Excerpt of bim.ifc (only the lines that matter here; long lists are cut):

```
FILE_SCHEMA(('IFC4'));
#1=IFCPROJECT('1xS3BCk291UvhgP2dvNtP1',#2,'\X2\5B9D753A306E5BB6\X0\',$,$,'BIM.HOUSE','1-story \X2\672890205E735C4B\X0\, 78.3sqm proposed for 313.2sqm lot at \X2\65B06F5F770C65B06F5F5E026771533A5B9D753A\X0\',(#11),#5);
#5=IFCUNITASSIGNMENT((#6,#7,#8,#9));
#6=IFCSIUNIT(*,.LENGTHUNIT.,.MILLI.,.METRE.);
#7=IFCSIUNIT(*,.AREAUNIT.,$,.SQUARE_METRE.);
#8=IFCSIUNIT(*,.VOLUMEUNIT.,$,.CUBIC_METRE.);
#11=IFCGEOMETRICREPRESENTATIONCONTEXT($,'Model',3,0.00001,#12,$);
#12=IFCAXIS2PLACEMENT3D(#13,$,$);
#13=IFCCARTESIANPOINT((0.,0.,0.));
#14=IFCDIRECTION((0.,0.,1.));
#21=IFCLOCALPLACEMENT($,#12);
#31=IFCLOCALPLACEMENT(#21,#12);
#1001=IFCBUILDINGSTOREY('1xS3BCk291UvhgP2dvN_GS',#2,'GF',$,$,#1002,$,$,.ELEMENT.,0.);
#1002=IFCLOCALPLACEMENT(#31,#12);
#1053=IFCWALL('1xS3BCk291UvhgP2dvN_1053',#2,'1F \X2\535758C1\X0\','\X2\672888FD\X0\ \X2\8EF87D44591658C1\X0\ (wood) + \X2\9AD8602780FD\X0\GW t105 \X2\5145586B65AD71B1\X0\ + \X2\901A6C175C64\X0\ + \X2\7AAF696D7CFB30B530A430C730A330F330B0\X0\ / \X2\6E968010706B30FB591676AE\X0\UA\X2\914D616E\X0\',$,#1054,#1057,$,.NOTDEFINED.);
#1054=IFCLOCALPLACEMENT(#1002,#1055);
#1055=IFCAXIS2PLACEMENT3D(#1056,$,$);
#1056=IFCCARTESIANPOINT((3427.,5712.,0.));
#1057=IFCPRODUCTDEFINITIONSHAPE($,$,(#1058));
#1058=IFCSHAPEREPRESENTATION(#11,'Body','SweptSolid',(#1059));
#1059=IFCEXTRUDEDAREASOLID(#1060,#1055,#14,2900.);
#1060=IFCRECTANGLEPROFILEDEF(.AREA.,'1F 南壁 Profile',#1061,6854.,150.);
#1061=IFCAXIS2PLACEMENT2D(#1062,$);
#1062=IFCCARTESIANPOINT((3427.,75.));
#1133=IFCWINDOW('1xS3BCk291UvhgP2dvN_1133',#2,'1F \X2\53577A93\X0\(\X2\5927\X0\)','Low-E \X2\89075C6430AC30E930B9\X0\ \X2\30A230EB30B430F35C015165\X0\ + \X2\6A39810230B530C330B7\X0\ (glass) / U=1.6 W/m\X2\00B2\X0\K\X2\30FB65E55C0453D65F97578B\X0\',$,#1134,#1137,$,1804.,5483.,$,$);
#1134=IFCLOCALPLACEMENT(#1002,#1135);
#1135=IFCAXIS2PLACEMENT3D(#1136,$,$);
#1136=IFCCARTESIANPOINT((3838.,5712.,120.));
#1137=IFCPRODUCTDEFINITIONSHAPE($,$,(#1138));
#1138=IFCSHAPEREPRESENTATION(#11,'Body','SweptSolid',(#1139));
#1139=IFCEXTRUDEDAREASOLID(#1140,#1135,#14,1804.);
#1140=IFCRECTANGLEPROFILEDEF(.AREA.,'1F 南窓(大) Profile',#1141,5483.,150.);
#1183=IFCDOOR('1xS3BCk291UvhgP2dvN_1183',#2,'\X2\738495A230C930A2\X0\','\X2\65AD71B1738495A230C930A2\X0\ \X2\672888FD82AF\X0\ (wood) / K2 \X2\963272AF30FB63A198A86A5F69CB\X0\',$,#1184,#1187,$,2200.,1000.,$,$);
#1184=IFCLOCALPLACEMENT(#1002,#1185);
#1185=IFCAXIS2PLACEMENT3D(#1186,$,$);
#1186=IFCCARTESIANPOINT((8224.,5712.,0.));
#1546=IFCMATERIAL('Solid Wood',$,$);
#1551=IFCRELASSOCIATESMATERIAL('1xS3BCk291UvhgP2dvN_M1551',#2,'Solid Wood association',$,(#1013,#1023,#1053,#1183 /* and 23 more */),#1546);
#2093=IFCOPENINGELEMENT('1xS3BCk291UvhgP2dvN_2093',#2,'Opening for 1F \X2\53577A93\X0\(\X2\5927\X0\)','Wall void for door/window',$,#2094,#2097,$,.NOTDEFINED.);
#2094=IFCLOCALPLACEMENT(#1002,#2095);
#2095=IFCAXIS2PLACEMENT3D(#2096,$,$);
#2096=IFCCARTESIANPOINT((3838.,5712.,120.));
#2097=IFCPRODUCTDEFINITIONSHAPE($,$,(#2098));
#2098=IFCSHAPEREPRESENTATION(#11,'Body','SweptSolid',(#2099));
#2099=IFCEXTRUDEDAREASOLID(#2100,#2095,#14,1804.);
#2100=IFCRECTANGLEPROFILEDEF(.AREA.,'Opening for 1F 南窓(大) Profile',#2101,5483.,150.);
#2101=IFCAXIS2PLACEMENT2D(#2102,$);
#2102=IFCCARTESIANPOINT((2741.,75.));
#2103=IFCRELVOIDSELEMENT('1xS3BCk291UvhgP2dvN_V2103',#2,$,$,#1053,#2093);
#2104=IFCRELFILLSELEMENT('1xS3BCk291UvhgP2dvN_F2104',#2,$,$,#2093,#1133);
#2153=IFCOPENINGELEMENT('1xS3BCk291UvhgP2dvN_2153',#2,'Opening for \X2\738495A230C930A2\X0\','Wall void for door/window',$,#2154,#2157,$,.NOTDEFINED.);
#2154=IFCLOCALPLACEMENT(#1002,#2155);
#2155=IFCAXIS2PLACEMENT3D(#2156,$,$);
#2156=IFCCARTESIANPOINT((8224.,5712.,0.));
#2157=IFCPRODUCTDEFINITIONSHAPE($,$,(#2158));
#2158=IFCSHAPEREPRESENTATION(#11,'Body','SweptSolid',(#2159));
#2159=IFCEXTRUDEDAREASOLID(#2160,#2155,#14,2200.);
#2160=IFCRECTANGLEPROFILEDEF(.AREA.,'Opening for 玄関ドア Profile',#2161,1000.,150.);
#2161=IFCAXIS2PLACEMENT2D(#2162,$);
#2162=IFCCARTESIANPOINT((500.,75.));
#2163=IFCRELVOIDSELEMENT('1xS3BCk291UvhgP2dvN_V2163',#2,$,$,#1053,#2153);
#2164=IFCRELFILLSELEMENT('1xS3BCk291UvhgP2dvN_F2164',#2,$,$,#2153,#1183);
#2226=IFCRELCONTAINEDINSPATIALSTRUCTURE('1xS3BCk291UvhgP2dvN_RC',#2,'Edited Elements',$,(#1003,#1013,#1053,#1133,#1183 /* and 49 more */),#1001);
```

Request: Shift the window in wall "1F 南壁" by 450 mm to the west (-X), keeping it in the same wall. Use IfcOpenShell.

```python
import ifcopenshell
import ifcopenshell.api.geometry
import ifcopenshell.util.placement
import ifcopenshell.util.unit

model = ifcopenshell.open("bim.ifc")
unit_scale = ifcopenshell.util.unit.calculate_unit_scale(model)

window = model.by_guid("1xS3BCk291UvhgP2dvN_1133")
opening = window.FillsVoids[0].RelatingOpeningElement
wall = opening.VoidsElements[0].RelatingBuildingElement

wall_matrix = ifcopenshell.util.placement.get_local_placement(wall.ObjectPlacement)
shift = wall_matrix[:3, 0] * -0.45 / unit_scale
before = ifcopenshell.util.placement.get_local_placement(window.ObjectPlacement)[:3, 3].copy()

# The window is not placed relative to its opening, so move both.
for product in (opening, window):
    matrix = ifcopenshell.util.placement.get_local_placement(product.ObjectPlacement)
    matrix[:3, 3] += shift
    ifcopenshell.api.geometry.edit_object_placement(model, product=product, matrix=matrix, is_si=False)

after = ifcopenshell.util.placement.get_local_placement(window.ObjectPlacement)[:3, 3]
print("window moved by", (after - before).round(3) + 0.0)

model.write("bim_edited.ifc")
```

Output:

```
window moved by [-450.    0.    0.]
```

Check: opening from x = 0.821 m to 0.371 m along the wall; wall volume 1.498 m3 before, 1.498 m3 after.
